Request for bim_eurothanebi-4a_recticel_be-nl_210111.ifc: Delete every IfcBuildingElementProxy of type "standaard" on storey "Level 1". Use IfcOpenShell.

First a look at what the model holds.

```python
import ifcopenshell
import ifcopenshell.util.element

model = ifcopenshell.open("bim_eurothanebi-4a_recticel_be-nl_210111.ifc")
print(model.schema)
storey = next(s for s in model.by_type("IfcBuildingStorey") if s.Name == "Level 1")
proxies = [e for e in ifcopenshell.util.element.get_decomposition(storey) if e.is_a("IfcBuildingElementProxy")]
seen = {}
for e in proxies:
    element_type = ifcopenshell.util.element.get_type(e)
    name = element_type.Name if element_type not in (None, e) else None
    seen[name] = seen.get(name, 0) + 1
for name, count in sorted(seen.items(), key=str):
    print(count, "x", name)
```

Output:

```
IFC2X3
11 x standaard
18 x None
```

```python
import ifcopenshell
import ifcopenshell.api.root
import ifcopenshell.util.element

model = ifcopenshell.open("bim_eurothanebi-4a_recticel_be-nl_210111.ifc")

storey = next(s for s in model.by_type("IfcBuildingStorey") if s.Name == "Level 1")
proxies = [e for e in ifcopenshell.util.element.get_decomposition(storey) if e.is_a("IfcBuildingElementProxy")]
targets = [e for e in proxies if (t := ifcopenshell.util.element.get_type(e)) not in (None, e) and t.Name == "standaard"]

for e in targets:
    ifcopenshell.api.root.remove_product(model, product=e)
print(len(targets), "removed")

model.write("bim_eurothanebi-4a_recticel_be-nl_210111_edited.ifc")
```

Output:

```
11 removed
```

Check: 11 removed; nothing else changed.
